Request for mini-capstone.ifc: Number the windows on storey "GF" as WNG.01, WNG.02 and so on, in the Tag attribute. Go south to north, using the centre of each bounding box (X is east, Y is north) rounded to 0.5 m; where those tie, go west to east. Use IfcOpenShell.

First a look at what the model holds.

```python
import ifcopenshell
import ifcopenshell.util.element
import ifcopenshell.util.placement

model = ifcopenshell.open("mini-capstone.ifc")
print(model.schema)
storey = next(s for s in model.by_type("IfcBuildingStorey") if s.Name == "GF")
windows = [e for e in ifcopenshell.util.element.get_decomposition(storey) if e.is_a("IfcWindow")]
for e in sorted(windows, key=lambda e: e.id()):
    origin = ifcopenshell.util.placement.get_local_placement(e.ObjectPlacement)[:3, 3]
    print(e.id(), e.Tag, e.Name, origin.round(2) + 0.0, sep=" | ")
```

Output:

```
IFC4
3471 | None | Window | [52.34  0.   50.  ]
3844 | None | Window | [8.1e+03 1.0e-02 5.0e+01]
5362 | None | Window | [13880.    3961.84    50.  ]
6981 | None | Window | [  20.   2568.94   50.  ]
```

```python
import ifcopenshell
import ifcopenshell.geom
import ifcopenshell.util.element
import ifcopenshell.util.shape

model = ifcopenshell.open("mini-capstone.ifc")
settings = ifcopenshell.geom.settings()
settings.set("use-world-coords", True)


def centre(element):
    shape = ifcopenshell.geom.create_shape(settings, element)
    return ifcopenshell.util.shape.get_bbox_centroid(shape.geometry)


storey = next(s for s in model.by_type("IfcBuildingStorey") if s.Name == "GF")
windows = [e for e in ifcopenshell.util.element.get_decomposition(storey) if e.is_a("IfcWindow")]

# Insertion points can sit at a corner or the storey origin, so sort by the geometry (in metres).
centres = {e: centre(e) for e in windows}
windows.sort(key=lambda e: (round(centres[e][1] / 0.5), centres[e][0]))

for i, e in enumerate(windows, start=1):
    number = f"WNG.{i:02d}"
    e.Tag = number
    print(e.id(), number)

model.write("mini-capstone_rev.ifc")
```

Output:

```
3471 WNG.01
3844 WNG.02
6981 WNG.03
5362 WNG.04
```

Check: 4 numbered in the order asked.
